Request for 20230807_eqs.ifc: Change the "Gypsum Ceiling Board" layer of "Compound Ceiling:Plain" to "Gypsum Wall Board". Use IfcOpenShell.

First a look at what the model holds.

```python
import ifcopenshell
import ifcopenshell.util.element

model = ifcopenshell.open("20230807_eqs.ifc")
print(model.schema)
for layer_set in model.by_type("IfcMaterialLayerSet"):
    if layer_set.LayerSetName == "Compound Ceiling:Plain":
        for layer in layer_set.MaterialLayers:
            print(layer.id(), layer.Material and layer.Material.Name, layer.LayerThickness, sep=" | ")
        print(len(ifcopenshell.util.element.get_elements_by_material(model, layer_set)), "elements and types use it")
print(sorted(m.Name for m in model.by_type("IfcMaterial") if m.Name)[:60])
```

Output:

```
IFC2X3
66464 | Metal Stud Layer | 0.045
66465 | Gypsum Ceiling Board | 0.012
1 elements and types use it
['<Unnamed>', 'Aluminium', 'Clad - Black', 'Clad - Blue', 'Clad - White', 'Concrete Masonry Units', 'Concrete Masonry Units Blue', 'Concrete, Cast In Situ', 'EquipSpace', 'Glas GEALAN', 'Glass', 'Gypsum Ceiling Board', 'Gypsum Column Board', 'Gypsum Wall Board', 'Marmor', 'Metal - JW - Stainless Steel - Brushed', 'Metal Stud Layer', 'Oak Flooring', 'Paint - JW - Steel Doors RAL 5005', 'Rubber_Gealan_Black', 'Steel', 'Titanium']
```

```python
import ifcopenshell
import ifcopenshell.api.material

model = ifcopenshell.open("20230807_eqs.ifc")

layer_set = next(s for s in model.by_type("IfcMaterialLayerSet") if s.LayerSetName == "Compound Ceiling:Plain")
layer = next(l for l in layer_set.MaterialLayers if l.Material and l.Material.Name == "Gypsum Ceiling Board")
material = next(m for m in model.by_type("IfcMaterial") if m.Name == "Gypsum Wall Board")

# Point this one layer at the other material; renaming the old one would change it everywhere.
ifcopenshell.api.material.edit_layer(model, layer=layer, attributes={}, material=material)

print([l.Material.Name if l.Material else None for l in layer_set.MaterialLayers])

model.write("20230807_eqs_rev.ifc")
```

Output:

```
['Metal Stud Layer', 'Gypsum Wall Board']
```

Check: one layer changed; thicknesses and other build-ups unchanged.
